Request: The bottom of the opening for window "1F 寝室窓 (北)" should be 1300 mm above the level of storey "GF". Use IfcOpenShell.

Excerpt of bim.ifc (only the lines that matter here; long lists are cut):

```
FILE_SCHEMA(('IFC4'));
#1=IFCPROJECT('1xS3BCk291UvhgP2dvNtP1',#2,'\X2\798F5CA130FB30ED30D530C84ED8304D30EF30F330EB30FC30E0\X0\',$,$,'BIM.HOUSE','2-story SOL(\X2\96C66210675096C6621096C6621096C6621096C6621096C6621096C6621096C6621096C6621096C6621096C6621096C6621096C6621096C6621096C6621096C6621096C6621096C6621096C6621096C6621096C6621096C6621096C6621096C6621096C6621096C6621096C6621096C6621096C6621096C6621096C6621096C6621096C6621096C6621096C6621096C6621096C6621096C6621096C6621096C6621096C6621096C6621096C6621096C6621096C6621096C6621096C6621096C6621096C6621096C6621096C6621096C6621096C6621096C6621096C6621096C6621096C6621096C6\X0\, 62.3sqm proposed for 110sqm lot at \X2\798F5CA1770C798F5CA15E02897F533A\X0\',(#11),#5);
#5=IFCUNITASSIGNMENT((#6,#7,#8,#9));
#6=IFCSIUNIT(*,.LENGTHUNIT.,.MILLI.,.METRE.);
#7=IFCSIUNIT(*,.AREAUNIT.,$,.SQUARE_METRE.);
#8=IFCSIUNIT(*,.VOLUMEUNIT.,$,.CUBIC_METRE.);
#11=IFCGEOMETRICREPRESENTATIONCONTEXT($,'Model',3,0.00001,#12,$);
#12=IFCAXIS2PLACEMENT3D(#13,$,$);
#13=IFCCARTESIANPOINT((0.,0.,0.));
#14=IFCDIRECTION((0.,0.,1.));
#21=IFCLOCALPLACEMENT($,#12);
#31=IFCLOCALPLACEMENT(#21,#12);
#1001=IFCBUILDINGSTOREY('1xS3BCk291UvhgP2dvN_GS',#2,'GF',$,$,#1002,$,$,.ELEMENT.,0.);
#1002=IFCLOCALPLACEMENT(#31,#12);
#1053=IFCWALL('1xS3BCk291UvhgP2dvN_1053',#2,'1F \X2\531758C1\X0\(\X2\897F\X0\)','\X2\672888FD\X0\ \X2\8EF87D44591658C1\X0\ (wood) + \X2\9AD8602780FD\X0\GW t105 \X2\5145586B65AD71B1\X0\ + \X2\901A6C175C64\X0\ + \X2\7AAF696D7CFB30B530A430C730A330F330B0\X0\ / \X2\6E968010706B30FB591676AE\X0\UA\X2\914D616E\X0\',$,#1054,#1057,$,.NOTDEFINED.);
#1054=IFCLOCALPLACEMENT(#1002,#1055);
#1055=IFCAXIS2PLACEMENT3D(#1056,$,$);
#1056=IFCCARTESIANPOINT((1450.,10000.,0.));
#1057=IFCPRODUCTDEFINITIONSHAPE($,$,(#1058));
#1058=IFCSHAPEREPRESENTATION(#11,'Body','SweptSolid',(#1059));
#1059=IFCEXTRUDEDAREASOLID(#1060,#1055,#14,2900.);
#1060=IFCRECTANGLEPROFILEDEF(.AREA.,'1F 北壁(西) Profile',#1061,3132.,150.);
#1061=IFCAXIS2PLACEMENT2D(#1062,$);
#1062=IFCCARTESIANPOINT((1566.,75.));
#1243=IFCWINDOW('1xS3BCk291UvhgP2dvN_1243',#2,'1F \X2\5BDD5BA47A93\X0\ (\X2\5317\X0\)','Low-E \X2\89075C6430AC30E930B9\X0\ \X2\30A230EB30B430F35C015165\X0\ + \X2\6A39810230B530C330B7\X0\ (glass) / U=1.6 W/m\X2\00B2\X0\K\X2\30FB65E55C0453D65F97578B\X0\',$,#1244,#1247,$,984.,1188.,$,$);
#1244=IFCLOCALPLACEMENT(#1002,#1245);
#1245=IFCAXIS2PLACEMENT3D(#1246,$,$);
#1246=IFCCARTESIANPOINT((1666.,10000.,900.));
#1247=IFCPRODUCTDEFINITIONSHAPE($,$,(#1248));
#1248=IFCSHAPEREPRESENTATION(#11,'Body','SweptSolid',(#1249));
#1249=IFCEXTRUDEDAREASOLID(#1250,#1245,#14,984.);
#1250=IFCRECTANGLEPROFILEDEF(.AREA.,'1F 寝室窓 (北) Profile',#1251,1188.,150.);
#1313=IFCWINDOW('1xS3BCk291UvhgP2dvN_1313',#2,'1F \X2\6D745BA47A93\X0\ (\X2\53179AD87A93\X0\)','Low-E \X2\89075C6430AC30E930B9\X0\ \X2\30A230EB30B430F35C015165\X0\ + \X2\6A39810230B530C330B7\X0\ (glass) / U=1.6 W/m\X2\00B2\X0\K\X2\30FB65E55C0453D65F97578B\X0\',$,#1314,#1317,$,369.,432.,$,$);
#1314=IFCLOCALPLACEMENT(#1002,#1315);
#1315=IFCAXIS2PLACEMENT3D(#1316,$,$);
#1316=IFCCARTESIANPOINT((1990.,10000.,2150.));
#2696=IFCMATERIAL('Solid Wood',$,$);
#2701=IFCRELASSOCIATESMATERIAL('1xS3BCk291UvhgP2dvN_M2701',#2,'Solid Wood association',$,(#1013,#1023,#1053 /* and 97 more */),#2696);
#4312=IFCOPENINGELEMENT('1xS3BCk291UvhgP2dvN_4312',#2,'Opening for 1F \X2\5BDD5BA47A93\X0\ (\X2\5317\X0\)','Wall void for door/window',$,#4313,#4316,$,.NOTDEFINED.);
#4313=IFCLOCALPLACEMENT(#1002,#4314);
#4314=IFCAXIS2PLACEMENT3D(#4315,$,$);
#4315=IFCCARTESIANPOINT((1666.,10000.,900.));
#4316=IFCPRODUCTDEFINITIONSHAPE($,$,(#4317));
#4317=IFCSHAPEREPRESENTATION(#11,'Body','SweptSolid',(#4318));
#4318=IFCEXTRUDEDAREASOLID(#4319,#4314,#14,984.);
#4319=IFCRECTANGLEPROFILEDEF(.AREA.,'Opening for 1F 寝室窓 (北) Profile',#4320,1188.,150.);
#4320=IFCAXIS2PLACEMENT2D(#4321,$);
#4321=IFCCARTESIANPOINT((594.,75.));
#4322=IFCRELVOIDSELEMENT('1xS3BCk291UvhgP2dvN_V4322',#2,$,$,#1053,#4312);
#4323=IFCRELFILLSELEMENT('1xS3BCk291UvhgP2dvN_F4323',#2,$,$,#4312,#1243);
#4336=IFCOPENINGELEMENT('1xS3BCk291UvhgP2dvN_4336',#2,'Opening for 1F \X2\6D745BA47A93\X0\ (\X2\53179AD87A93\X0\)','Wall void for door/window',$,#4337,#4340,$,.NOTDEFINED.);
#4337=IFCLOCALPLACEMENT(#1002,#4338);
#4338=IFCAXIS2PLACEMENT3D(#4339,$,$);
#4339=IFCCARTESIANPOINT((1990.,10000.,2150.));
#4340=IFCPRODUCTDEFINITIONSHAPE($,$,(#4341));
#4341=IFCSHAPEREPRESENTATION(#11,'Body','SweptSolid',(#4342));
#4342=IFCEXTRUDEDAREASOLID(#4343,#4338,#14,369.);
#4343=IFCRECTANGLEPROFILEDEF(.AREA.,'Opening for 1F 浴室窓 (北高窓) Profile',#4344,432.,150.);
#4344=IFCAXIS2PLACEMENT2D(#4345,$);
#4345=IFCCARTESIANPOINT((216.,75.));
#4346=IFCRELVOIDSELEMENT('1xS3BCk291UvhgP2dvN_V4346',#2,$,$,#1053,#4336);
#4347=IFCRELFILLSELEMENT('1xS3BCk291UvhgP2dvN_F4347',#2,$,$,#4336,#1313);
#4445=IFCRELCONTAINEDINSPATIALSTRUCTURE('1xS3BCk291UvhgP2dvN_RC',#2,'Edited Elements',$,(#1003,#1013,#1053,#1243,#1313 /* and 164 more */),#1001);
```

```python
import numpy as np
import ifcopenshell
import ifcopenshell.api.geometry
import ifcopenshell.geom
import ifcopenshell.util.element
import ifcopenshell.util.placement
import ifcopenshell.util.shape
import ifcopenshell.util.unit

model = ifcopenshell.open("bim.ifc")
unit_scale = ifcopenshell.util.unit.calculate_unit_scale(model)

window = model.by_id(1243)
opening = window.FillsVoids[0].RelatingOpeningElement
storey = ifcopenshell.util.element.get_container(window, ifc_class="IfcBuildingStorey")
level = ifcopenshell.util.placement.get_local_placement(storey.ObjectPlacement)[2, 3]

# The opening's origin need not be at the sill, so measure its lowest point.
shape = ifcopenshell.geom.create_shape(ifcopenshell.geom.settings(), opening)
bottom = ifcopenshell.util.shape.get_shape_bottom_elevation(shape, shape.geometry) / unit_scale
dz = level + 1.3 / unit_scale - bottom

shift = np.array([0.0, 0.0, dz])
# The window is not placed relative to its opening, so move both.
for product in (opening, window):
    matrix = ifcopenshell.util.placement.get_local_placement(product.ObjectPlacement)
    matrix[:3, 3] += shift
    ifcopenshell.api.geometry.edit_object_placement(model, product=product, matrix=matrix, is_si=False)

print(f"moved by {dz * unit_scale:+.3f} m")

model.write("bim-out.ifc")
```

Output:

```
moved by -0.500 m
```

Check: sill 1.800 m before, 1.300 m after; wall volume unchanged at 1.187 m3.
